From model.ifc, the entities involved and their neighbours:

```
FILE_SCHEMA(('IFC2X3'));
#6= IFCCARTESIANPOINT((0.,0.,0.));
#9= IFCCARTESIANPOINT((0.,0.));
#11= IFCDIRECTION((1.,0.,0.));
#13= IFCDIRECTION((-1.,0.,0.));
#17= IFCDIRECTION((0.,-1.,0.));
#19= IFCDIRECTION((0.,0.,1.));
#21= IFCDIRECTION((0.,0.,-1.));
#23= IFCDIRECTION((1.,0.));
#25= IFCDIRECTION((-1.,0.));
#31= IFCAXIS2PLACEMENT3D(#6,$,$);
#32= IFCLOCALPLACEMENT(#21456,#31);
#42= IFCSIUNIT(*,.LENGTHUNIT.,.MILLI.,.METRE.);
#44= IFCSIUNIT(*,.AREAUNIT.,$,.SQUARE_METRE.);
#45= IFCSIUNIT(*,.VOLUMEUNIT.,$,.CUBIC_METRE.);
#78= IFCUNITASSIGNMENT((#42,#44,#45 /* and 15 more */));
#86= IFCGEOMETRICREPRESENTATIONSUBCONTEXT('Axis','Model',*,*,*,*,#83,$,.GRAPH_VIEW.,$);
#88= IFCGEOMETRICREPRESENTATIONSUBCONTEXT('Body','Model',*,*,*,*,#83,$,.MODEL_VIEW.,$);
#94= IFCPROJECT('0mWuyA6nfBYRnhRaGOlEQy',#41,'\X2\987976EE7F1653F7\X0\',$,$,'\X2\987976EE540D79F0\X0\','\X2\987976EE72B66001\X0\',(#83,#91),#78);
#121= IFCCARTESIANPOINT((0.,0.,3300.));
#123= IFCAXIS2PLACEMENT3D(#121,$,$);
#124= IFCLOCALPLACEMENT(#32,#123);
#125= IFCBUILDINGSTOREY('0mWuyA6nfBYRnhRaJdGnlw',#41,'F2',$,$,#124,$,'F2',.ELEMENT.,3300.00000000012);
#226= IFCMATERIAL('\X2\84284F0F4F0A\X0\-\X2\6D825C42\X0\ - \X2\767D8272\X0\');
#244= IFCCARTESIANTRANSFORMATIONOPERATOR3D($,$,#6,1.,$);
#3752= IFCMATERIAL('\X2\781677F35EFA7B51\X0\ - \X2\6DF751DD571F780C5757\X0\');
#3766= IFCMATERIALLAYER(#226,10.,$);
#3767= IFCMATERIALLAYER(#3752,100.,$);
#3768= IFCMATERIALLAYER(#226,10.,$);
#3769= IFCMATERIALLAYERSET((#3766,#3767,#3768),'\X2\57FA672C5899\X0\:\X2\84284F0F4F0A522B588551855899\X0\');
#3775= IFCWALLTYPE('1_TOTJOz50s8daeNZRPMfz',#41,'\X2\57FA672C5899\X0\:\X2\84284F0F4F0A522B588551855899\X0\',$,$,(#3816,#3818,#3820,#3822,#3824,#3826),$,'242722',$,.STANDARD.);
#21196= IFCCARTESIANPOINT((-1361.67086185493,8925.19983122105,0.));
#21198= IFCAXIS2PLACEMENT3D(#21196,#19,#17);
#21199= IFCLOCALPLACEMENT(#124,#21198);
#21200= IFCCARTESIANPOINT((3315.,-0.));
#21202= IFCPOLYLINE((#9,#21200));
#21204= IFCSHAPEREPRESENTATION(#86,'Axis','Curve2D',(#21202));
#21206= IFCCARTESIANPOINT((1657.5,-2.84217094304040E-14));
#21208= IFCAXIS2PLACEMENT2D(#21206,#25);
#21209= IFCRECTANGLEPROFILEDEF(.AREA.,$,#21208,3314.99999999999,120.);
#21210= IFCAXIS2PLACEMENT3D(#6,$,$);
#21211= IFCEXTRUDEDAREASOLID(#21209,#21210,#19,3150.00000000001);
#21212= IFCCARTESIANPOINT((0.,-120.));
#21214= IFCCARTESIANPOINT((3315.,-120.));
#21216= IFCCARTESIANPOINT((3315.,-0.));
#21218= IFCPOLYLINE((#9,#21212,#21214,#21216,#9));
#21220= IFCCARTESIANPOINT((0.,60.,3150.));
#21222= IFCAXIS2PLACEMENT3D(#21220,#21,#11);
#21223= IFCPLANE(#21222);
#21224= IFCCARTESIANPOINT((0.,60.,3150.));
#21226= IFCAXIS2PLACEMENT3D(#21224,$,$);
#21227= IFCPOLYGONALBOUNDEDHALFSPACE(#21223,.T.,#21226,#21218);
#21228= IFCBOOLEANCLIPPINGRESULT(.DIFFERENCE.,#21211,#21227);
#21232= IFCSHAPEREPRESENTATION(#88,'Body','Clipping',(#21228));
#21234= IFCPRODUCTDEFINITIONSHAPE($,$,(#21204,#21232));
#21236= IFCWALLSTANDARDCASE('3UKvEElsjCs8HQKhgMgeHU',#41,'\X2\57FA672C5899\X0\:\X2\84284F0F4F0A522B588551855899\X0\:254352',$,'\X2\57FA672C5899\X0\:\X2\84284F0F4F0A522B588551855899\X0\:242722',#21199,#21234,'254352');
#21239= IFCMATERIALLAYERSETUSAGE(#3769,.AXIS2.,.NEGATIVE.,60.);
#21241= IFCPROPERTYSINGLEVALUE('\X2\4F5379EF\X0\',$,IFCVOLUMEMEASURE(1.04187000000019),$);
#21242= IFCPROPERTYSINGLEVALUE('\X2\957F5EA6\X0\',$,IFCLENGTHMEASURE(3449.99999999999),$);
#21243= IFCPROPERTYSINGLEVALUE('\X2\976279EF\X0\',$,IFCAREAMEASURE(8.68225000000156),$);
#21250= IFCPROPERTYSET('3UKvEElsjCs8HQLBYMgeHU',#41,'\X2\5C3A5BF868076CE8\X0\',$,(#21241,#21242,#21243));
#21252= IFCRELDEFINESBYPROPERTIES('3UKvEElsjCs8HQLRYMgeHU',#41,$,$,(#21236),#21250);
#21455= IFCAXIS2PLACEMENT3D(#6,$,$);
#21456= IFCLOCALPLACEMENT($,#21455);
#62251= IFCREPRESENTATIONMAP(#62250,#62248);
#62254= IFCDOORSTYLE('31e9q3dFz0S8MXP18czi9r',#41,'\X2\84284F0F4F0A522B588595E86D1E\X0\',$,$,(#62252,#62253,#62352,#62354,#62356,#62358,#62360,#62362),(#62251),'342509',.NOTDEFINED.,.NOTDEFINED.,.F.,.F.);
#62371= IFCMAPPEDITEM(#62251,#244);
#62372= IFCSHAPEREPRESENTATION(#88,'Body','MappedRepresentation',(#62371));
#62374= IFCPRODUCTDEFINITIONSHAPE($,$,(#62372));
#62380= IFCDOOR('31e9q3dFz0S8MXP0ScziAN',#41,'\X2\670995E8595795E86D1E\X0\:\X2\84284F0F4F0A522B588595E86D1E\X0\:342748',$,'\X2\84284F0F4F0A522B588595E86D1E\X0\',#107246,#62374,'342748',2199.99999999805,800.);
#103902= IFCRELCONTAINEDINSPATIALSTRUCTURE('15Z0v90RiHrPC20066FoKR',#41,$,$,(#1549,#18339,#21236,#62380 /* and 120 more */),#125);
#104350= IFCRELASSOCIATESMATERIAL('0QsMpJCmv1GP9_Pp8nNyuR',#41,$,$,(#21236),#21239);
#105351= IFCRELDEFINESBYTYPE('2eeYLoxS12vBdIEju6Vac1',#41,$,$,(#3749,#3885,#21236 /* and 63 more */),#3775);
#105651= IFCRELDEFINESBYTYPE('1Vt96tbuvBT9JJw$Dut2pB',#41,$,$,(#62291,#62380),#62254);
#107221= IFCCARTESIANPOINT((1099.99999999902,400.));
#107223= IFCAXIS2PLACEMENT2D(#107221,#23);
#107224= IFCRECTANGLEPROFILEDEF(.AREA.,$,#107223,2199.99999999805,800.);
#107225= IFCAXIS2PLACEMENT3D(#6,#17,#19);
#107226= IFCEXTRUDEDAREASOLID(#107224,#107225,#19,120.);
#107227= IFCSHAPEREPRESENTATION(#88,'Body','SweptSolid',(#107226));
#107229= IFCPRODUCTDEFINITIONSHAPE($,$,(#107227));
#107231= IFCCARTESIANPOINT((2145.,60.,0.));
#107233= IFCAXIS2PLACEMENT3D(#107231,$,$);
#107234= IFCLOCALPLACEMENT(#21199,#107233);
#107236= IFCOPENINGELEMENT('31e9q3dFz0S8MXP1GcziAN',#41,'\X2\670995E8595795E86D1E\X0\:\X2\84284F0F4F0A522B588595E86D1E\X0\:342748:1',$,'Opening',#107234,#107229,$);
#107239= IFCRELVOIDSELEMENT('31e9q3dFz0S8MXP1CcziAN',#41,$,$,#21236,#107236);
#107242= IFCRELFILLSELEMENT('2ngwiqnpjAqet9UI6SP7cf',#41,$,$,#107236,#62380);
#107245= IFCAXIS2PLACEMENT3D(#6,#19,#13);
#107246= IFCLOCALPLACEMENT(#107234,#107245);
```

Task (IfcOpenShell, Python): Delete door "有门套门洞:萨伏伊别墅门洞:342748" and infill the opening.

```python
import ifcopenshell
import ifcopenshell.api.feature
import ifcopenshell.api.pset
import ifcopenshell.api.root
import ifcopenshell.geom
import ifcopenshell.util.element
import ifcopenshell.util.shape
import ifcopenshell.util.unit

model = ifcopenshell.open("model.ifc")
area_scale = ifcopenshell.util.unit.calculate_unit_scale(model, "AREAUNIT")
volume_scale = ifcopenshell.util.unit.calculate_unit_scale(model, "VOLUMEUNIT")
settings = ifcopenshell.geom.settings()


def volume(element):
    """Net volume in cubic metres, openings subtracted."""
    shape = ifcopenshell.geom.create_shape(settings, element)
    return ifcopenshell.util.shape.get_volume(shape.geometry)


door = model.by_id(62380)
opening = door.FillsVoids[0].RelatingOpeningElement
wall = opening.VoidsElements[0].RelatingBuildingElement
before = volume(wall)

ifcopenshell.api.root.remove_product(model, product=door)
ifcopenshell.api.feature.remove_feature(model, feature=opening)

after = volume(wall)
thickness = 0.12  # wall thickness in metres

# Update the wall's stored quantities.
pset = model.by_id(ifcopenshell.util.element.get_pset(wall, "尺寸标注", should_inherit=False)["id"])
ifcopenshell.api.pset.edit_pset(model, pset=pset, properties={
    "体积": model.create_entity("IfcVolumeMeasure", after / volume_scale),
    "面积": model.create_entity("IfcAreaMeasure", after / thickness / area_scale),
})

print(f"wall volume {before:.3f} -> {after:.3f} m3")

model.write("model_v2.ifc")
```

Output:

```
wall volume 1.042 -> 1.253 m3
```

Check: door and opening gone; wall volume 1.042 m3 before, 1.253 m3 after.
